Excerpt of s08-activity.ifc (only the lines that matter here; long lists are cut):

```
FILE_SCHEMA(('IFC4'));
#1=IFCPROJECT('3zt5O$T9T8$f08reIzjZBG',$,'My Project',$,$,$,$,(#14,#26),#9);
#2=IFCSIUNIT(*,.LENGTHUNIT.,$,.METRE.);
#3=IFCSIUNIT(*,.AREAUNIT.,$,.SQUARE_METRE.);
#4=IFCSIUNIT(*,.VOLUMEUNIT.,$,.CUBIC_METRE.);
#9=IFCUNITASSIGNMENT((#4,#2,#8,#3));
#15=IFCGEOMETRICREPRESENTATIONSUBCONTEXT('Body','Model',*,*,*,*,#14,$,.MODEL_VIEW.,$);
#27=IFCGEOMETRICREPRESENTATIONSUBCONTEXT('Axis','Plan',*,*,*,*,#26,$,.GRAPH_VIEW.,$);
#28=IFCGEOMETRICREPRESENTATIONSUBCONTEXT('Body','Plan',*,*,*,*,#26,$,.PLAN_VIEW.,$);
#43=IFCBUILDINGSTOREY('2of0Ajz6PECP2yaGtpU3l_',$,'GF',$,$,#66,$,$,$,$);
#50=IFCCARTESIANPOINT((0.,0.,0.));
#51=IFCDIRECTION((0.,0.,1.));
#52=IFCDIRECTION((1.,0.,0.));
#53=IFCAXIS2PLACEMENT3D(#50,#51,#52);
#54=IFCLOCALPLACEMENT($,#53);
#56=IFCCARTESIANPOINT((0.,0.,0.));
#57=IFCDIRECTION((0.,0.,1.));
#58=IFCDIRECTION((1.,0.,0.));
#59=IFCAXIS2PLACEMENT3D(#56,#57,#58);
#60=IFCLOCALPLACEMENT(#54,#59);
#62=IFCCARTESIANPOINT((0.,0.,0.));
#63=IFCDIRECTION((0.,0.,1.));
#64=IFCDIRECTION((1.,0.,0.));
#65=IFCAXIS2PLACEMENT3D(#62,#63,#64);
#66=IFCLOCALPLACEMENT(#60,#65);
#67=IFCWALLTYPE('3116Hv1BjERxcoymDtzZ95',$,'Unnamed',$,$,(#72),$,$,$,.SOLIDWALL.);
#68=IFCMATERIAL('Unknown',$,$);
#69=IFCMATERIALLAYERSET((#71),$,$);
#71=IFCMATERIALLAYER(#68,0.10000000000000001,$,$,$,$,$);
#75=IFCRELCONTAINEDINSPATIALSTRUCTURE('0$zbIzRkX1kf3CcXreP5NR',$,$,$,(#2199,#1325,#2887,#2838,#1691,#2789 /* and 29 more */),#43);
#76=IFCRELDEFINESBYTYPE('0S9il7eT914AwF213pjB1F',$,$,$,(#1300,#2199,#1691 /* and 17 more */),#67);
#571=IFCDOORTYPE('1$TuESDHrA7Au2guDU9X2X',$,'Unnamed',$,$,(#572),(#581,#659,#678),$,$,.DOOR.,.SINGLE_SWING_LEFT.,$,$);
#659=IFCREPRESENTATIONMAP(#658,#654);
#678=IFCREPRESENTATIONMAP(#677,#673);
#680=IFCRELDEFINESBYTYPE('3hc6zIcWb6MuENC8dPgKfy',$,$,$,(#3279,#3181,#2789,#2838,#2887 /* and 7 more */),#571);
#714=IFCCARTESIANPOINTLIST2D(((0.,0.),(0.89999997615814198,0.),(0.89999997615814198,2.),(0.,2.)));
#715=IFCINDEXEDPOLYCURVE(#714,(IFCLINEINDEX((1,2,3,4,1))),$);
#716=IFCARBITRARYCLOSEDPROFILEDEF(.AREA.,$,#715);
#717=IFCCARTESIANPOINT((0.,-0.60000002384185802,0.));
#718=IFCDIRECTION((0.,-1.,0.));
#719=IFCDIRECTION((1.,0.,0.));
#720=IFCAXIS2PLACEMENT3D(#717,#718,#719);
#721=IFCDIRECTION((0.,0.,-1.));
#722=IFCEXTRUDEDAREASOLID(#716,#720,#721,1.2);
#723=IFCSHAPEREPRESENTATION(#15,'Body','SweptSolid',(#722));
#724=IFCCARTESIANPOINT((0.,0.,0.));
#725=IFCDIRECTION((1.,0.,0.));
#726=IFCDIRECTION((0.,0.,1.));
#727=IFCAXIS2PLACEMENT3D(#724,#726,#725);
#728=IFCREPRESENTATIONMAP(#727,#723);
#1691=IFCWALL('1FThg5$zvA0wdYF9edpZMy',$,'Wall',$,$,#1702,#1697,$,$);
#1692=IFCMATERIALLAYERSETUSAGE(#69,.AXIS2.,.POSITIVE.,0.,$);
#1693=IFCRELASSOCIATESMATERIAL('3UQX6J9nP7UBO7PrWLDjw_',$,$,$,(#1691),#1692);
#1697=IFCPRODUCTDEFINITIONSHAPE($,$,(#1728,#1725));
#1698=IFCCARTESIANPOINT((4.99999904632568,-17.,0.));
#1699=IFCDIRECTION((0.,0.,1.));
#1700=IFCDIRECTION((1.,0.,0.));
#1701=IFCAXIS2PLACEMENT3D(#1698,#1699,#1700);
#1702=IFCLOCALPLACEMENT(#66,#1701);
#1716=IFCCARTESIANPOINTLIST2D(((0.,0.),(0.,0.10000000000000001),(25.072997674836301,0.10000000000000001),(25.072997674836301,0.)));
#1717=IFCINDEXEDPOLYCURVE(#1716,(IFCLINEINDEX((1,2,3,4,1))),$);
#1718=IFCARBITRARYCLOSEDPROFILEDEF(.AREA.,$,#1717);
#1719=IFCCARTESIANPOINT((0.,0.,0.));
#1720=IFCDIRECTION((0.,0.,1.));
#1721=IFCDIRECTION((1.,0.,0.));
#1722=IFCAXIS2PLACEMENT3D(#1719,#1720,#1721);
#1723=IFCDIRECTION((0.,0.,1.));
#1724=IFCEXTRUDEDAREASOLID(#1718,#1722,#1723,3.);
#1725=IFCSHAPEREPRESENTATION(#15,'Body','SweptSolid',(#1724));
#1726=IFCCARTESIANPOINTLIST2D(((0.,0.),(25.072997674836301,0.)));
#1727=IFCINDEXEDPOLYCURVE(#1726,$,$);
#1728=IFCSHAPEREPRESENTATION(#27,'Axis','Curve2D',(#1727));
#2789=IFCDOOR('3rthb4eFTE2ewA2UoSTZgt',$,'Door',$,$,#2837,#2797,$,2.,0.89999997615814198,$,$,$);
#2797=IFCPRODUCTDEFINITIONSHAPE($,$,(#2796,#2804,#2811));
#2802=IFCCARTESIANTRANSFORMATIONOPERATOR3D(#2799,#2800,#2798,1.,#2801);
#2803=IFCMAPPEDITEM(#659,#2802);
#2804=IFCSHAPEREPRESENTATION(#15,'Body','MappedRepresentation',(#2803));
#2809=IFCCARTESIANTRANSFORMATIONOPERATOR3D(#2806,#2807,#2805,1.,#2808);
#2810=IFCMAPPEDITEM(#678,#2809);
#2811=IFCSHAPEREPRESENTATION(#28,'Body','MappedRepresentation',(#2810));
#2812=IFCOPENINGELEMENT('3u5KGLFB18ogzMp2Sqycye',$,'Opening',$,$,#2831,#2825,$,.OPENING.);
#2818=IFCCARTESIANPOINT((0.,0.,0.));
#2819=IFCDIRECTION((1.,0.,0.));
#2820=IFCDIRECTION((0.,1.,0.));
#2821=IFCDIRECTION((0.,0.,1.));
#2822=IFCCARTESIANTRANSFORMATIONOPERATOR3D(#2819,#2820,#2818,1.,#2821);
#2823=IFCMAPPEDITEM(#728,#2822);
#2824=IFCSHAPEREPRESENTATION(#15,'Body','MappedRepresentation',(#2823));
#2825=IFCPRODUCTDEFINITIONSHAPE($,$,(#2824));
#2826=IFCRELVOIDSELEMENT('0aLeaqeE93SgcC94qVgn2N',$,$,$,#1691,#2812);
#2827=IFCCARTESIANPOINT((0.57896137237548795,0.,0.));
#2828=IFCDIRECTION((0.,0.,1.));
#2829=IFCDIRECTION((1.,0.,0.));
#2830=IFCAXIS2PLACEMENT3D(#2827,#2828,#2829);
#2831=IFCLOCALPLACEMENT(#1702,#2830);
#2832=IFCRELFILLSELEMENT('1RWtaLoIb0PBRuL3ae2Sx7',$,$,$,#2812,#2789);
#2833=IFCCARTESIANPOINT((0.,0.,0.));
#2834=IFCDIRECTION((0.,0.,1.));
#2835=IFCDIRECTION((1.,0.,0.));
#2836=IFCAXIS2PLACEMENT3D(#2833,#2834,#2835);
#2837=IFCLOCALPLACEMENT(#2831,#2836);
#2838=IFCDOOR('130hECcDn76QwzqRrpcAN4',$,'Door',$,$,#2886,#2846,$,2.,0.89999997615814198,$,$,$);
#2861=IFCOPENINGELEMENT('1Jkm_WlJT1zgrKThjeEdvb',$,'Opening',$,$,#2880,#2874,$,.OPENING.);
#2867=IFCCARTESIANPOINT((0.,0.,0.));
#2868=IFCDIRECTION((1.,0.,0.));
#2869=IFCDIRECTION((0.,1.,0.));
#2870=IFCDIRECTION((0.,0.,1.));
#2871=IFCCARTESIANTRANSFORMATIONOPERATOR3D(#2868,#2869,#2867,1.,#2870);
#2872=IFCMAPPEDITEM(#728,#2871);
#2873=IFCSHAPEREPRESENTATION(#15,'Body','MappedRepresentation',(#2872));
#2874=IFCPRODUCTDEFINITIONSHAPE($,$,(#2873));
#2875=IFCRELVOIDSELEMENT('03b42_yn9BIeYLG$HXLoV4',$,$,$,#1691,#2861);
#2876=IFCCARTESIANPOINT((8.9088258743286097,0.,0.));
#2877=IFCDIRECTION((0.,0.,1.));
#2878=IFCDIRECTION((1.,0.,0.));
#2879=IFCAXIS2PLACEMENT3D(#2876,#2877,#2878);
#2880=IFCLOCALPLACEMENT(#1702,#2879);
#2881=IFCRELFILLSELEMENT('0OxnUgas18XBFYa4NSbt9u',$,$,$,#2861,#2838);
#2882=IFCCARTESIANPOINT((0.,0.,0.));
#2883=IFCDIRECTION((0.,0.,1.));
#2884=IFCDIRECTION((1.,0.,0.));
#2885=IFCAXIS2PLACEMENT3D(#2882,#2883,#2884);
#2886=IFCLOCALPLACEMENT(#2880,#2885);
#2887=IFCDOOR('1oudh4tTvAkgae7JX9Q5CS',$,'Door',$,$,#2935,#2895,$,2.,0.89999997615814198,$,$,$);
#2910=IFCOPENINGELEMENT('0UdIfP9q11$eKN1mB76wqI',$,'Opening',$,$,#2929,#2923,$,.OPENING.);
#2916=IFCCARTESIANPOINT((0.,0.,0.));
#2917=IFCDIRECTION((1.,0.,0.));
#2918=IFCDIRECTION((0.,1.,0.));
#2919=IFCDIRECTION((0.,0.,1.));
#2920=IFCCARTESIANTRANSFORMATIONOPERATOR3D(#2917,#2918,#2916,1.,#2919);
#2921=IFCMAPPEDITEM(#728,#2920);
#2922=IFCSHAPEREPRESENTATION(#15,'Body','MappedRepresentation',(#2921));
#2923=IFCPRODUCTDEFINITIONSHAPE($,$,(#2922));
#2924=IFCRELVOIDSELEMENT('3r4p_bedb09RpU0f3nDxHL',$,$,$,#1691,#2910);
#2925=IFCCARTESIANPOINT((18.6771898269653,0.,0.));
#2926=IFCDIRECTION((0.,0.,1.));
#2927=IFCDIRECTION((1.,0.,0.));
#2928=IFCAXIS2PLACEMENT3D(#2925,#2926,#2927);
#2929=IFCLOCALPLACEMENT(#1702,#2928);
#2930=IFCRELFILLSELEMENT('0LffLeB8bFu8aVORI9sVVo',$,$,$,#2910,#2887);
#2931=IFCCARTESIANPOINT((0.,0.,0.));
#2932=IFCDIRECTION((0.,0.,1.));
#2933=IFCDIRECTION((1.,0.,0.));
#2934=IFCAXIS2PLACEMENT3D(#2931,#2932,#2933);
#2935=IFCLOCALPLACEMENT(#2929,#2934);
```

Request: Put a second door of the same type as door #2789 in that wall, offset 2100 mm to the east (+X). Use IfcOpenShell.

```python
import ifcopenshell
import ifcopenshell.api.feature
import ifcopenshell.api.geometry
import ifcopenshell.api.root
import ifcopenshell.geom
import ifcopenshell.util.element
import ifcopenshell.util.placement
import ifcopenshell.util.shape
import ifcopenshell.util.unit

model = ifcopenshell.open("s08-activity.ifc")
unit_scale = ifcopenshell.util.unit.calculate_unit_scale(model)
settings = ifcopenshell.geom.settings()


def volume(element):
    """Net volume in cubic metres, openings subtracted."""
    shape = ifcopenshell.geom.create_shape(settings, element)
    return ifcopenshell.util.shape.get_volume(shape.geometry)


door = model.by_guid("3rthb4eFTE2ewA2UoSTZgt")
opening = door.FillsVoids[0].RelatingOpeningElement
wall = opening.VoidsElements[0].RelatingBuildingElement
before = volume(wall)
shift = ifcopenshell.util.placement.get_local_placement(wall.ObjectPlacement)[:3, 0] * 2.1 / unit_scale

# copy_class copies the void relationship, type, container and properties, but no geometry.
new_opening = ifcopenshell.api.root.copy_class(model, product=opening)
new_opening.Representation = ifcopenshell.util.element.copy_deep(
    model, opening.Representation, exclude=["IfcGeometricRepresentationContext", "IfcRepresentationMap"]
)
new_door = ifcopenshell.api.root.copy_class(model, product=door)
new_door.Representation = ifcopenshell.util.element.copy_deep(
    model, door.Representation, exclude=["IfcGeometricRepresentationContext", "IfcRepresentationMap"]
)
ifcopenshell.api.feature.add_filling(model, opening=new_opening, element=new_door)

for old, new in ((opening, new_opening), (door, new_door)):
    matrix = ifcopenshell.util.placement.get_local_placement(old.ObjectPlacement)
    matrix[:3, 3] += shift
    ifcopenshell.api.geometry.edit_object_placement(model, product=new, matrix=matrix, is_si=False)

after = volume(wall)

print(f"wall volume {before:.3f} -> {after:.3f} m3")

model.write("s08-activity-out.ifc")
```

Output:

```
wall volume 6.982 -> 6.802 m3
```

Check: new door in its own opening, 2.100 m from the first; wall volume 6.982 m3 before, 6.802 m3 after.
